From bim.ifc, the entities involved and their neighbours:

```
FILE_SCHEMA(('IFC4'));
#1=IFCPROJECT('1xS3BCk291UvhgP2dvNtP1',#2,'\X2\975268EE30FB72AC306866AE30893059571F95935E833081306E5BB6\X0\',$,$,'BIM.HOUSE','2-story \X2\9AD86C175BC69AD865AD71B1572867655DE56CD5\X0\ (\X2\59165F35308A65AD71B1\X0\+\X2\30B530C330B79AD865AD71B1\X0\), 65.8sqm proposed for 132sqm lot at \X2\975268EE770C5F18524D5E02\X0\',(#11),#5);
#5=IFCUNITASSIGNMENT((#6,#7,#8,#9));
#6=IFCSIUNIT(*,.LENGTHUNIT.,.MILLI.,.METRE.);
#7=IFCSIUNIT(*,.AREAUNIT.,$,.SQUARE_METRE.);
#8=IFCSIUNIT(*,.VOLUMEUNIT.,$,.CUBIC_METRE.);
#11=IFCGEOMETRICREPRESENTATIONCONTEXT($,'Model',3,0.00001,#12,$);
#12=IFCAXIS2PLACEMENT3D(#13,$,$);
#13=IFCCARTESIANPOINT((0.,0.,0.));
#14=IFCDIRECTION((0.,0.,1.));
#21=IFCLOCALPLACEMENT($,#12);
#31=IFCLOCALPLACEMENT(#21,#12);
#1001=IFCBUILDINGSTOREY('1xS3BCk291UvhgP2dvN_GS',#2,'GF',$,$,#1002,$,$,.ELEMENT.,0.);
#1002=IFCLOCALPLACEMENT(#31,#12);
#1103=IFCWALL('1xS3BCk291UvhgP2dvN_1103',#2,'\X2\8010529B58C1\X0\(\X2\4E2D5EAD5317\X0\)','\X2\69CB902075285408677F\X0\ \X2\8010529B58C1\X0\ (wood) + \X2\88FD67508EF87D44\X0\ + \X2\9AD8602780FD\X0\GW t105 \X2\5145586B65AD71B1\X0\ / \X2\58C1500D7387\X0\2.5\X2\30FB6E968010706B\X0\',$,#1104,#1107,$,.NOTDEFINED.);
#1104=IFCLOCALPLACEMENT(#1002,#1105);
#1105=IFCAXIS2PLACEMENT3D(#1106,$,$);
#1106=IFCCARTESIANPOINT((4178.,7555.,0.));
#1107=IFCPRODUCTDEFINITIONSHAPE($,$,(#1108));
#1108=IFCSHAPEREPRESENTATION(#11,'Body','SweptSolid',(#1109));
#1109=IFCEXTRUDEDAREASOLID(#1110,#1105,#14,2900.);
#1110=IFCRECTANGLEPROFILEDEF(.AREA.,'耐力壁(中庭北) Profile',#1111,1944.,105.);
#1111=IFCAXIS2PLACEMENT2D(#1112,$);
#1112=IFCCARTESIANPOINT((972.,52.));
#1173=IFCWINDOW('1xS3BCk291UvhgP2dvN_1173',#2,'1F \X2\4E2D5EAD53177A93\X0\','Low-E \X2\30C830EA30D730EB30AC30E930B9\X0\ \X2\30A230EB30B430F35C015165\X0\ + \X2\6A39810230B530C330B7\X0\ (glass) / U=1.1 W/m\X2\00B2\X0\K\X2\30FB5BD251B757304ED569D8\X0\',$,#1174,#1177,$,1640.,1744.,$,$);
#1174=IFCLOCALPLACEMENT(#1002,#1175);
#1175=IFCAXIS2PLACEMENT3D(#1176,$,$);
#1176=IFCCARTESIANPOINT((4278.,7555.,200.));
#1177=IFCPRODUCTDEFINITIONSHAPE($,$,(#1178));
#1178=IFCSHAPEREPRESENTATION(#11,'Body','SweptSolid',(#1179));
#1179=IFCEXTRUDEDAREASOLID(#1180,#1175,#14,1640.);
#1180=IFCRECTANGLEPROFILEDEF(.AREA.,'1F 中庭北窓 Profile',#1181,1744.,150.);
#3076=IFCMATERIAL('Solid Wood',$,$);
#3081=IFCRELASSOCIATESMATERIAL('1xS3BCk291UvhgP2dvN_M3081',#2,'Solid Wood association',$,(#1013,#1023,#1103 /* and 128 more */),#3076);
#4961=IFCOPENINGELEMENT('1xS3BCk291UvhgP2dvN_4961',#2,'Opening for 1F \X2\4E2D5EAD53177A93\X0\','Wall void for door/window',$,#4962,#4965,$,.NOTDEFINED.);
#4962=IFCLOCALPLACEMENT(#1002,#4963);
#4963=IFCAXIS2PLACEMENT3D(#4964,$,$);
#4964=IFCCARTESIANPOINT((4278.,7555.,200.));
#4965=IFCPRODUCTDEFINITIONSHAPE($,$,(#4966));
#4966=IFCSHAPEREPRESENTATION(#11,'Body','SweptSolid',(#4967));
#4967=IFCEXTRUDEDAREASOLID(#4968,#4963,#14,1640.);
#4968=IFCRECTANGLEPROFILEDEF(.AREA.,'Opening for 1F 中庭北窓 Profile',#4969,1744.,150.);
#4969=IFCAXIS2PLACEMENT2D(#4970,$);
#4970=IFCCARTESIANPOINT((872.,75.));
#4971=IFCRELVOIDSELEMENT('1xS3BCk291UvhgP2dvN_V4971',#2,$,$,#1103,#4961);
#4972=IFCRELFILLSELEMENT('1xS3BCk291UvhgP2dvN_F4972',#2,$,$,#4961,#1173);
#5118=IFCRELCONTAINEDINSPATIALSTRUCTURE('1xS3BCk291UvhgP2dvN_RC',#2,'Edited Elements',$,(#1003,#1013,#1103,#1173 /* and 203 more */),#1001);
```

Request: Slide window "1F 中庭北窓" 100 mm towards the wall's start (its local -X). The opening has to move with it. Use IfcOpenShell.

```python
import ifcopenshell
import ifcopenshell.api.geometry
import ifcopenshell.util.placement

model = ifcopenshell.open("bim.ifc")

window = model.by_guid("1xS3BCk291UvhgP2dvN_1173")
opening = window.FillsVoids[0].RelatingOpeningElement
wall = opening.VoidsElements[0].RelatingBuildingElement

wall_matrix = ifcopenshell.util.placement.get_local_placement(wall.ObjectPlacement)
shift = wall_matrix[:3, 0] * -100.0
before = ifcopenshell.util.placement.get_local_placement(window.ObjectPlacement)[:3, 3].copy()

# The window is not placed relative to its opening, so move both.
for product in (opening, window):
    matrix = ifcopenshell.util.placement.get_local_placement(product.ObjectPlacement)
    matrix[:3, 3] += shift
    ifcopenshell.api.geometry.edit_object_placement(model, product=product, matrix=matrix, is_si=False)

after = ifcopenshell.util.placement.get_local_placement(window.ObjectPlacement)[:3, 3]
print("window moved by", (after - before).round(3) + 0.0)

model.write("bim_v2.ifc")
```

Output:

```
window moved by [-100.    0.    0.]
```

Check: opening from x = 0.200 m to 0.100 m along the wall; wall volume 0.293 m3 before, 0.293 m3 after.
